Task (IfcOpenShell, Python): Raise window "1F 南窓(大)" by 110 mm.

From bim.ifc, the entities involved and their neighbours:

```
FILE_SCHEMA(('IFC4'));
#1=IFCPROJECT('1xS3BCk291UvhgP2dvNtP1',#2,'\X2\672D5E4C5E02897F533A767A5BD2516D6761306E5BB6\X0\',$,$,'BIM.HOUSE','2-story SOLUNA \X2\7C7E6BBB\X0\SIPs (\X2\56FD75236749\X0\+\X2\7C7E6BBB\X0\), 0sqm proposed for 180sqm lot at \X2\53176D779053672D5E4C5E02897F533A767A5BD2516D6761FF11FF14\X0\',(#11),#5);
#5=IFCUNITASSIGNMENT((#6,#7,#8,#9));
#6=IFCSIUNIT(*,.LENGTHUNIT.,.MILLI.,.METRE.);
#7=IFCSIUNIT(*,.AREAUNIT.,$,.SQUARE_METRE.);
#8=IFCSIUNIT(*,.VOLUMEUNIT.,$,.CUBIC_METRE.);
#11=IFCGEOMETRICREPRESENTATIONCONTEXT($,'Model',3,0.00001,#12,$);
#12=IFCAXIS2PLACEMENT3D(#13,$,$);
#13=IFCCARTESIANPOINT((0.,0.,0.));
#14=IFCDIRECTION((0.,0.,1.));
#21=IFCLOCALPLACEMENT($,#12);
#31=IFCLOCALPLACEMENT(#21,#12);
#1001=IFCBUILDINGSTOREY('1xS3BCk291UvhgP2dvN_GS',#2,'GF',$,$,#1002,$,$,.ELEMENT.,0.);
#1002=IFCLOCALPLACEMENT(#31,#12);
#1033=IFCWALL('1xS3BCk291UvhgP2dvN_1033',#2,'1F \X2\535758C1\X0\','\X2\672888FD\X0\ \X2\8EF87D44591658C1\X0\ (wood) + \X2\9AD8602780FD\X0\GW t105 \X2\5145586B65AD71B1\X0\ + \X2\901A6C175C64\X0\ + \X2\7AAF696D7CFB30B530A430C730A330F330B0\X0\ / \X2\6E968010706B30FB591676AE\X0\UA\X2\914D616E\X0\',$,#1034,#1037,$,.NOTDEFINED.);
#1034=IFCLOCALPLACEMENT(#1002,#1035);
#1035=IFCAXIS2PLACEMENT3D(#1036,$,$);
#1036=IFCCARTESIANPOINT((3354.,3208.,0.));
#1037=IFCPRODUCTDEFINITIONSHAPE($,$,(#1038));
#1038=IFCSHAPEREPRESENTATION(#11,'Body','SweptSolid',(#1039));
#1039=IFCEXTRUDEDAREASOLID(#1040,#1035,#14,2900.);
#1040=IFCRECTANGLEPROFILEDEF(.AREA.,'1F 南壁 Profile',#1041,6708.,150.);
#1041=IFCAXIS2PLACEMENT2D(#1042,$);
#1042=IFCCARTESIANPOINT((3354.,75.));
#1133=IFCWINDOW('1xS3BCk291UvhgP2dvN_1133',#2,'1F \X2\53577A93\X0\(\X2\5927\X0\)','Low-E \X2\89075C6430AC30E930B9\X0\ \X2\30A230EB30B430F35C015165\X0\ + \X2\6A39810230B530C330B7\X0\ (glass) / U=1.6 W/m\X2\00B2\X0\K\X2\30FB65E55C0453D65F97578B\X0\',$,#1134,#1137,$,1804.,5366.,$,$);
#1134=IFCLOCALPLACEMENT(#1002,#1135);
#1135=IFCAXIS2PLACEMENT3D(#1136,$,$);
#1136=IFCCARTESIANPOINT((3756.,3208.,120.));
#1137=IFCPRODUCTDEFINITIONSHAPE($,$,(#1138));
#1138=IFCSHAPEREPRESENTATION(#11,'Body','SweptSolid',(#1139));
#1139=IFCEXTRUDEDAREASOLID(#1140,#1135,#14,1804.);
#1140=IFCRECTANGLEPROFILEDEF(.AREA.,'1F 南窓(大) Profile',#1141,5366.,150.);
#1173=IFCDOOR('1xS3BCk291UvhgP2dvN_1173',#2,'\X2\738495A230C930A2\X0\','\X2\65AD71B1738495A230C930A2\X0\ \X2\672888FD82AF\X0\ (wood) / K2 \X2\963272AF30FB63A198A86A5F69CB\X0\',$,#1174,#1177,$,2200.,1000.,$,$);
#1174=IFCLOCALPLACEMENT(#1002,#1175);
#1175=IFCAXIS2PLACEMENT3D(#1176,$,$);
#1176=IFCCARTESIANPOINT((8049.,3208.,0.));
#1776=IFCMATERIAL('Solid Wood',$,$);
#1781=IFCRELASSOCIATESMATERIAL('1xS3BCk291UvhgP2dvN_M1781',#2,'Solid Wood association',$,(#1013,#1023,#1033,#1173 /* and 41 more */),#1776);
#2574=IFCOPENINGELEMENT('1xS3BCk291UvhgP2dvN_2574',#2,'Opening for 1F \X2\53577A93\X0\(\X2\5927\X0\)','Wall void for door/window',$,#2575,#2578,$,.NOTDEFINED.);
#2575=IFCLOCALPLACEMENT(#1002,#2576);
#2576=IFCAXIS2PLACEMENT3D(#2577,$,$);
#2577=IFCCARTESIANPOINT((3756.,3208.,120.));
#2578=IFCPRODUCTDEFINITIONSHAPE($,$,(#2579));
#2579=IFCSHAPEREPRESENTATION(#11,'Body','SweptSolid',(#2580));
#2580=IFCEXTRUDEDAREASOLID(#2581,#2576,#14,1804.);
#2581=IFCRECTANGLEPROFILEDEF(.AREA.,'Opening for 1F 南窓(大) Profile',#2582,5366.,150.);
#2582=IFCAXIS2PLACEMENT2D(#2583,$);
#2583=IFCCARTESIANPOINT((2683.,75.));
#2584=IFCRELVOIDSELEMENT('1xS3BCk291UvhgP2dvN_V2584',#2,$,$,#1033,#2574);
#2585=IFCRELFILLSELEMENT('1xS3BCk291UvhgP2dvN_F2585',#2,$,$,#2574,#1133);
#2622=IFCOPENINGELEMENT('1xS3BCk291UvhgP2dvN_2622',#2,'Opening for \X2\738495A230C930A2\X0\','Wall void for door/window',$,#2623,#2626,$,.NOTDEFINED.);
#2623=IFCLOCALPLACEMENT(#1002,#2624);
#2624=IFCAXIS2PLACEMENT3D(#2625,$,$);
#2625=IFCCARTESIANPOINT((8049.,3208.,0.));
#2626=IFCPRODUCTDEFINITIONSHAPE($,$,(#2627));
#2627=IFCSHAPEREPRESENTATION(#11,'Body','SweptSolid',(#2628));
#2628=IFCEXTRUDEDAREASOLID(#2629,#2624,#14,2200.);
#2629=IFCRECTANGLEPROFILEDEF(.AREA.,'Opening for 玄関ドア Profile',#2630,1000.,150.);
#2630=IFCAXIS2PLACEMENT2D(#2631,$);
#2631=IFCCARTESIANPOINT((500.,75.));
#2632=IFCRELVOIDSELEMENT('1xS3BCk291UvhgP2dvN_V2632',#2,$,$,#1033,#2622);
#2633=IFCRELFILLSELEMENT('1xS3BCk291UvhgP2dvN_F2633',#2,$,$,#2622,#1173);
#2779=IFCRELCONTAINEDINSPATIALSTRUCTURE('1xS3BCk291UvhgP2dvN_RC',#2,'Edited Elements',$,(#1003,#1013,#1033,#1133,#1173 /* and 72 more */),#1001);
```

```python
import numpy as np
import ifcopenshell
import ifcopenshell.api.geometry
import ifcopenshell.util.placement
import ifcopenshell.util.unit

model = ifcopenshell.open("bim.ifc")
unit_scale = ifcopenshell.util.unit.calculate_unit_scale(model)

window = model.by_guid("1xS3BCk291UvhgP2dvN_1133")
opening = window.FillsVoids[0].RelatingOpeningElement
dz = 0.11 / unit_scale

shift = np.array([0.0, 0.0, dz])
# The window is not placed relative to its opening, so move both.
for product in (opening, window):
    matrix = ifcopenshell.util.placement.get_local_placement(product.ObjectPlacement)
    matrix[:3, 3] += shift
    ifcopenshell.api.geometry.edit_object_placement(model, product=product, matrix=matrix, is_si=False)

print(f"moved by {dz * unit_scale:+.3f} m")

model.write("bim_rev.ifc")
```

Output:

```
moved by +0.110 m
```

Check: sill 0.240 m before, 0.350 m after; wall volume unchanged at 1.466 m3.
